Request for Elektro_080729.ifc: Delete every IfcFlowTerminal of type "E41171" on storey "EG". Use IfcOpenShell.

First a look at what the model holds.

```python
import ifcopenshell
import ifcopenshell.util.element

model = ifcopenshell.open("Elektro_080729.ifc")
print(model.schema)
storey = next(s for s in model.by_type("IfcBuildingStorey") if s.Name == "EG")
terminals = [e for e in ifcopenshell.util.element.get_decomposition(storey) if e.is_a("IfcFlowTerminal")]
seen = {}
for e in terminals:
    element_type = ifcopenshell.util.element.get_type(e)
    name = element_type.Name if element_type not in (None, e) else None
    seen[name] = seen.get(name, 0) + 1
for name, count in sorted(seen.items(), key=str):
    print(count, "x", name)
```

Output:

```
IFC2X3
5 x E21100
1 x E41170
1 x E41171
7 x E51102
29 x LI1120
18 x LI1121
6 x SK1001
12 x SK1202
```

```python
import ifcopenshell
import ifcopenshell.api.root
import ifcopenshell.util.element

model = ifcopenshell.open("Elektro_080729.ifc")

storey = next(s for s in model.by_type("IfcBuildingStorey") if s.Name == "EG")
terminals = [e for e in ifcopenshell.util.element.get_decomposition(storey) if e.is_a("IfcFlowTerminal")]
targets = [e for e in terminals if (t := ifcopenshell.util.element.get_type(e)) not in (None, e) and t.Name == "E41171"]

for e in targets:
    ifcopenshell.api.root.remove_product(model, product=e)
print(len(targets), "removed")

model.write("Elektro_080729_edited.ifc")
```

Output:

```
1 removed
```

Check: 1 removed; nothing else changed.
